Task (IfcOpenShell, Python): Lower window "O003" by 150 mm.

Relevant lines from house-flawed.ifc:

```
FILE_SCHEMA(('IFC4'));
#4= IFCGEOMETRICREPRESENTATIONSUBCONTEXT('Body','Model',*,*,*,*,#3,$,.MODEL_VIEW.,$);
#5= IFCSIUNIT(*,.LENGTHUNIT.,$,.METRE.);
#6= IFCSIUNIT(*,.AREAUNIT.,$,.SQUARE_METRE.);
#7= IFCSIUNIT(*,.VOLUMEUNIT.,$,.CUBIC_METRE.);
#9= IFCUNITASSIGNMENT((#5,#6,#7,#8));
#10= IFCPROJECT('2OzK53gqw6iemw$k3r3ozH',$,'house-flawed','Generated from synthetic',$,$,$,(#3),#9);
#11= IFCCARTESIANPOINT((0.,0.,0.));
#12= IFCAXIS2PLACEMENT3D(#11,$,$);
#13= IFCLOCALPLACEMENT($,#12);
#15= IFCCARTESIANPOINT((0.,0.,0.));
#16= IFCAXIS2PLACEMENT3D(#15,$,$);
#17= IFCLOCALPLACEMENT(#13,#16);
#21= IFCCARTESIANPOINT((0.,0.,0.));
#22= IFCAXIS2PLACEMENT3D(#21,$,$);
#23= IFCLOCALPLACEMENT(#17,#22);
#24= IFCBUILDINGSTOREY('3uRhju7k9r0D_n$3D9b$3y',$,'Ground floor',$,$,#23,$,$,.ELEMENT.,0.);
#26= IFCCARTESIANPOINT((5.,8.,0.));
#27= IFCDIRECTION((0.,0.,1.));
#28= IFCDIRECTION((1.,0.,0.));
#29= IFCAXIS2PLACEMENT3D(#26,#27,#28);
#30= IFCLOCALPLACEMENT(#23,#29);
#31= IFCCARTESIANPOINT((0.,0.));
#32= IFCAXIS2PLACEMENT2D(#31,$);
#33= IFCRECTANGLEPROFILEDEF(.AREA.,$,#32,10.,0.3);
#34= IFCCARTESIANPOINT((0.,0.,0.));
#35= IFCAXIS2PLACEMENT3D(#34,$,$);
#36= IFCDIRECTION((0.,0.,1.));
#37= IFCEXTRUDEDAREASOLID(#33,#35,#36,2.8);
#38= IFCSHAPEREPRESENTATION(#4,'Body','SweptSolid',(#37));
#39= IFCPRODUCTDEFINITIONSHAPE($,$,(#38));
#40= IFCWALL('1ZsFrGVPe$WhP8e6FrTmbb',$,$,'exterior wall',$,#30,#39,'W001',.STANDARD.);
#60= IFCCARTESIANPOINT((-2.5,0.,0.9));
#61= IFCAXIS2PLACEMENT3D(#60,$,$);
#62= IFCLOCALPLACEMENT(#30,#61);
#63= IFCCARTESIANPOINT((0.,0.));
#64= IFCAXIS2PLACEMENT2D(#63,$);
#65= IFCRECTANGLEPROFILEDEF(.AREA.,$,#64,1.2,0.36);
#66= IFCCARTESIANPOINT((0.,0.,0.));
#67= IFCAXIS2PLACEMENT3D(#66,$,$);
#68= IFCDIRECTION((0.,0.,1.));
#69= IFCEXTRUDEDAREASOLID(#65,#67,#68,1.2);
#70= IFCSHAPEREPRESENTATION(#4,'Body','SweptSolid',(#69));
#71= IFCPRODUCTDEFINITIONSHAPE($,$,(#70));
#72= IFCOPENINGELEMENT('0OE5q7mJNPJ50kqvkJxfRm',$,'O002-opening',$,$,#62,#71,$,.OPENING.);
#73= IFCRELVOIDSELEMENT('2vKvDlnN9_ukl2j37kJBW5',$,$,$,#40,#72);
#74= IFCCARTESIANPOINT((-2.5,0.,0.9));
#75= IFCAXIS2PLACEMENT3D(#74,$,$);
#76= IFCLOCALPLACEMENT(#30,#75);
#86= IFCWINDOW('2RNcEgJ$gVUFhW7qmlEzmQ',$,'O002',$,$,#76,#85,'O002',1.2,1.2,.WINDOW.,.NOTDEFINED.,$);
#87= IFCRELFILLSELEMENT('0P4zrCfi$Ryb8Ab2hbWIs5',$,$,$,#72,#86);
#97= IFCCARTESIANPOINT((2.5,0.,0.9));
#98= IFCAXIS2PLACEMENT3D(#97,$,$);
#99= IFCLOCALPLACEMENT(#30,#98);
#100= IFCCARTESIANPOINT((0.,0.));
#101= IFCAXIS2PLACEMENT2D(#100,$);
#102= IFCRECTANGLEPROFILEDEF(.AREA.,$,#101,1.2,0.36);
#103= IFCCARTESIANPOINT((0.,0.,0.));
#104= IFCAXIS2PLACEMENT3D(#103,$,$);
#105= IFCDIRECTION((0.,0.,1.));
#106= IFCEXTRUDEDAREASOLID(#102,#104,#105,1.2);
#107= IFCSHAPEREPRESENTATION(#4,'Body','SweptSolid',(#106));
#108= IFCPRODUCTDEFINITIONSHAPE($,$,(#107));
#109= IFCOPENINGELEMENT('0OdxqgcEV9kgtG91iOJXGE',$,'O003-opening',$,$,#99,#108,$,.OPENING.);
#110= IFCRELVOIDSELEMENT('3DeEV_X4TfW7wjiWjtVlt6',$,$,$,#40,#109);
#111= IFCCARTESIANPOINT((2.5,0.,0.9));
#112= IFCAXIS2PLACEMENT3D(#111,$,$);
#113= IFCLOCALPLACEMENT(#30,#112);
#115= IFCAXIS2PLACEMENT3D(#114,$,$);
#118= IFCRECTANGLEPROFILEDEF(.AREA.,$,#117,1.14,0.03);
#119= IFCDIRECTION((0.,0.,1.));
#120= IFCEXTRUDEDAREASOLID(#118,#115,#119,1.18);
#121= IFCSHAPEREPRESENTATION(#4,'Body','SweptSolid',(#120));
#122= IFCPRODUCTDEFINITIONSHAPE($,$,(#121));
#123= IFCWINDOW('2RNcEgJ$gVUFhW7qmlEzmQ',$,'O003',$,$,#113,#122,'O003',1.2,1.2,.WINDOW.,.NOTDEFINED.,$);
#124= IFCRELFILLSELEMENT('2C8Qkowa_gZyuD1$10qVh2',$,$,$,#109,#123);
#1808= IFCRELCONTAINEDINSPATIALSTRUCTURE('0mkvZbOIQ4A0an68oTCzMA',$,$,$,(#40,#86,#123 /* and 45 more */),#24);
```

```python
import numpy as np
import ifcopenshell
import ifcopenshell.api.geometry
import ifcopenshell.util.placement
import ifcopenshell.util.unit

model = ifcopenshell.open("house-flawed.ifc")
unit_scale = ifcopenshell.util.unit.calculate_unit_scale(model)

window = model.by_guid("2RNcEgJ$gVUFhW7qmlEzmQ")
opening = window.FillsVoids[0].RelatingOpeningElement
dz = -0.15 / unit_scale

shift = np.array([0.0, 0.0, dz])
# The window is not placed relative to its opening, so move both.
for product in (opening, window):
    matrix = ifcopenshell.util.placement.get_local_placement(product.ObjectPlacement)
    matrix[:3, 3] += shift
    ifcopenshell.api.geometry.edit_object_placement(model, product=product, matrix=matrix, is_si=False)

print(f"moved by {dz * unit_scale:+.3f} m")

model.write("house-flawed_updated.ifc")
```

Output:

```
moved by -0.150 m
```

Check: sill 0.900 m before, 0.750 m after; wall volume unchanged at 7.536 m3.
